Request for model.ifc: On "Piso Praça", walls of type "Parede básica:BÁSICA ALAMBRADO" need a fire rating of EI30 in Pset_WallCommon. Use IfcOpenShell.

First a look at what the model holds.

```python
import ifcopenshell
import ifcopenshell.util.element

model = ifcopenshell.open("model.ifc")
print(model.schema)
storey = next(s for s in model.by_type("IfcBuildingStorey") if s.Name == "Piso Praça")
walls = [e for e in ifcopenshell.util.element.get_decomposition(storey) if e.is_a("IfcWall")]
seen = {}
for e in walls:
    element_type = ifcopenshell.util.element.get_type(e)
    key = (element_type.Name if element_type != e and element_type else None, ifcopenshell.util.element.get_pset(e, "Pset_WallCommon", "FireRating"))
    seen[key] = seen.get(key, 0) + 1
for (name, value), count in sorted(seen.items(), key=str):
    print(count, "x", name, "|", value)
```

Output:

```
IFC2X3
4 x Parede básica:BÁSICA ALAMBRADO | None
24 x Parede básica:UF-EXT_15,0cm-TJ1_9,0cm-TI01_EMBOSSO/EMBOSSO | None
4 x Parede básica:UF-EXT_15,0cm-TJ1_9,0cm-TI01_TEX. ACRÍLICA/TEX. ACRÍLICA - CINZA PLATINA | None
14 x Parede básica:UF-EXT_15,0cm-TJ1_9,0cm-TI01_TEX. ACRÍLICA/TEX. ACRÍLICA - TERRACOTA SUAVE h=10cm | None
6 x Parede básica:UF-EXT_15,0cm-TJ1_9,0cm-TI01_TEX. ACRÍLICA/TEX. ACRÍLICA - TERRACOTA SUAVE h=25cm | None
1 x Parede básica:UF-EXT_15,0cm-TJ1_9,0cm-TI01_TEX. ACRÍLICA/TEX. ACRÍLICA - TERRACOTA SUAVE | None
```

```python
import ifcopenshell
import ifcopenshell.api.pset
import ifcopenshell.util.element

model = ifcopenshell.open("model.ifc")

storey = next(s for s in model.by_type("IfcBuildingStorey") if s.Name == "Piso Praça")
walls = [e for e in ifcopenshell.util.element.get_decomposition(storey) if e.is_a("IfcWall")]

count = 0
for e in walls:
    element_type = ifcopenshell.util.element.get_type(e)
    if element_type in (None, e) or element_type.Name != "Parede básica:BÁSICA ALAMBRADO":
        continue
    # add_pset returns the element's existing set when there is one.
    pset = ifcopenshell.api.pset.add_pset(model, product=e, name="Pset_WallCommon")
    ifcopenshell.api.pset.edit_pset(model, pset=pset, properties={"FireRating": "EI30"})
    count += 1

print(count, "walls updated")

model.write("model_updated.ifc")
```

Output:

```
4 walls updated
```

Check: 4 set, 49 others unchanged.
